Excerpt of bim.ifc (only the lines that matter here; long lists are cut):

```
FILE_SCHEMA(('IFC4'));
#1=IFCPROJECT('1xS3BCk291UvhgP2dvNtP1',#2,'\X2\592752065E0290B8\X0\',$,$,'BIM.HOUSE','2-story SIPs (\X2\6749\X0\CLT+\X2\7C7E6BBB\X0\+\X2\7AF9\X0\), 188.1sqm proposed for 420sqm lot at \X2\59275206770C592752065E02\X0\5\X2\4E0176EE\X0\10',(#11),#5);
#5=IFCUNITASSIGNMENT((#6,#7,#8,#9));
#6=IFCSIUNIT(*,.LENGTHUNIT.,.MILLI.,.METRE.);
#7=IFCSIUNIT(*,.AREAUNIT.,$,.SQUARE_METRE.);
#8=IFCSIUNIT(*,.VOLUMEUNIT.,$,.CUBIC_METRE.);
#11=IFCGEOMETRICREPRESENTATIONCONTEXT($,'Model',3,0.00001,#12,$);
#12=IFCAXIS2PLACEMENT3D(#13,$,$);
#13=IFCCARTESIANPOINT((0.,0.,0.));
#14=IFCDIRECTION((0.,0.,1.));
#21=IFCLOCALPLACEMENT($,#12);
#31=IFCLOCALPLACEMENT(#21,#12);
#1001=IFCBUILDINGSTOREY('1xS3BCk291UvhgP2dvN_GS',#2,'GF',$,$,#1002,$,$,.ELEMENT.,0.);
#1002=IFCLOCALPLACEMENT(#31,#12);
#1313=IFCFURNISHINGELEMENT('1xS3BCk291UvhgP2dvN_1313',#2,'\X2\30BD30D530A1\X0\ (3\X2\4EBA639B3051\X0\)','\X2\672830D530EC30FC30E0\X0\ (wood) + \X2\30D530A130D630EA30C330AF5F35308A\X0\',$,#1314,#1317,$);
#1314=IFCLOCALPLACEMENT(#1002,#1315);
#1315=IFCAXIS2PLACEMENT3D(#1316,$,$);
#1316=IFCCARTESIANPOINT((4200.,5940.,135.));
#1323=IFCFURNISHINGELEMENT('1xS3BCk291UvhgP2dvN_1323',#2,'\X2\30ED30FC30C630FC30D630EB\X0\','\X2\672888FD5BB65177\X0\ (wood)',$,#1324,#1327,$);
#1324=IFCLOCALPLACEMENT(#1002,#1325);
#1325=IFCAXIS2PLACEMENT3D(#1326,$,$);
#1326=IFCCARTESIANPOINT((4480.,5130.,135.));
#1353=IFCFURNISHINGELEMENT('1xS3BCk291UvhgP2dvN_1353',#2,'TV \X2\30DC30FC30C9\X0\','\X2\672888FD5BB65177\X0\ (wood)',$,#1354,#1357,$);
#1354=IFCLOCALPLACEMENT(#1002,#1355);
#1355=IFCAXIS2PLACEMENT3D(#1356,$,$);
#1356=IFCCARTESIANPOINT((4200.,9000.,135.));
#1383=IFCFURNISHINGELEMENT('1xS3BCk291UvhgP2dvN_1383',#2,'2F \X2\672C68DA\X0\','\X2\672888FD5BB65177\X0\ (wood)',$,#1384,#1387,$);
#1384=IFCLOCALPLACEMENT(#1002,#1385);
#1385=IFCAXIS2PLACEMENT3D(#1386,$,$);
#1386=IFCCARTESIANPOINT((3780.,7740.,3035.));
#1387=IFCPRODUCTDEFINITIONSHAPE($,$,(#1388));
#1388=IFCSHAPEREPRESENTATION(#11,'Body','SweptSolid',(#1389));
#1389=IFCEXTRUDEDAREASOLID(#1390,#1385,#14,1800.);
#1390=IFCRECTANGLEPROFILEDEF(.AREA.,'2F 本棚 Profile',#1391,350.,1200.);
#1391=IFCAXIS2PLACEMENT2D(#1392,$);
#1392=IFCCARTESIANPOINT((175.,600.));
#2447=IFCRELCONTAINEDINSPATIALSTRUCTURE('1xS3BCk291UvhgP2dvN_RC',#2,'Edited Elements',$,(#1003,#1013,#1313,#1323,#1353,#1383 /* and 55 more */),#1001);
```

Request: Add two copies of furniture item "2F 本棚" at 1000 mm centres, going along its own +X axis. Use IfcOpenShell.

```python
import ifcopenshell
import ifcopenshell.api.geometry
import ifcopenshell.api.root
import ifcopenshell.util.element
import ifcopenshell.util.placement

model = ifcopenshell.open("bim.ifc")


def reuse_history(source, copy):
    """copy_class also copies each property set's owner history, people and application; keep the originals."""
    for rel in copy.IsDefinedBy:
        if rel.is_a("IfcRelDefinesByProperties") and (history := rel.RelatingPropertyDefinition.OwnerHistory):
            rel.RelatingPropertyDefinition.OwnerHistory = source.OwnerHistory
            ifcopenshell.util.element.remove_deep2(model, history)


source = model.by_guid("1xS3BCk291UvhgP2dvN_1383")
base = ifcopenshell.util.placement.get_local_placement(source.ObjectPlacement)
step = base[:3, 0] * 1000.0

for i in range(1, 3):
    copy = ifcopenshell.api.root.copy_class(model, product=source)
    copy.Representation = ifcopenshell.util.element.copy_deep(
        model, source.Representation, exclude=["IfcGeometricRepresentationContext", "IfcRepresentationMap"]
    )
    reuse_history(source, copy)
    matrix = base.copy()
    matrix[:3, 3] += i * step
    print("added at", matrix[:3, 3].round(3) + 0.0)
    ifcopenshell.api.geometry.edit_object_placement(model, product=copy, matrix=matrix, is_si=False)

model.write("bim-out.ifc")
```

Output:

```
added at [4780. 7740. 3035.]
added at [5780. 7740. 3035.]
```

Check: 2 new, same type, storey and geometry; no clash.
